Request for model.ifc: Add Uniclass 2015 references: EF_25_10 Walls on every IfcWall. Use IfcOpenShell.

First a look at what the model holds.

```python
import ifcopenshell

model = ifcopenshell.open("model.ifc")
print(model.schema)
print("classifications:", [c.Name for c in model.by_type("IfcClassification")])
for ifc_class in ("IfcDoor", "IfcRoof", "IfcStair", "IfcWall", "IfcWindow"):
    print(ifc_class, len(model.by_type(ifc_class)))
```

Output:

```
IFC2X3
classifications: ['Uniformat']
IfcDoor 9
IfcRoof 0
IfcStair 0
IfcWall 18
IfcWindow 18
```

```python
import ifcopenshell
import ifcopenshell.api.classification

model = ifcopenshell.open("model.ifc")

# IFC2X3 requires Source and Edition and has no link from the project to the system.
system = model.create_entity("IfcClassification", Source="NBS", Edition="2015", Name="Uniclass 2015")

codes = {
    "IfcWall": ("EF_25_10", "Walls"),
}
for ifc_class, (code, name) in codes.items():
    products = model.by_type(ifc_class)
    ifcopenshell.api.classification.add_reference(
        model, products=products, classification=system, identification=code, name=name
    )
    print(code, len(products))

model.write("model-out.ifc")
```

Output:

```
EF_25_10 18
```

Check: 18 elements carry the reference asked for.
